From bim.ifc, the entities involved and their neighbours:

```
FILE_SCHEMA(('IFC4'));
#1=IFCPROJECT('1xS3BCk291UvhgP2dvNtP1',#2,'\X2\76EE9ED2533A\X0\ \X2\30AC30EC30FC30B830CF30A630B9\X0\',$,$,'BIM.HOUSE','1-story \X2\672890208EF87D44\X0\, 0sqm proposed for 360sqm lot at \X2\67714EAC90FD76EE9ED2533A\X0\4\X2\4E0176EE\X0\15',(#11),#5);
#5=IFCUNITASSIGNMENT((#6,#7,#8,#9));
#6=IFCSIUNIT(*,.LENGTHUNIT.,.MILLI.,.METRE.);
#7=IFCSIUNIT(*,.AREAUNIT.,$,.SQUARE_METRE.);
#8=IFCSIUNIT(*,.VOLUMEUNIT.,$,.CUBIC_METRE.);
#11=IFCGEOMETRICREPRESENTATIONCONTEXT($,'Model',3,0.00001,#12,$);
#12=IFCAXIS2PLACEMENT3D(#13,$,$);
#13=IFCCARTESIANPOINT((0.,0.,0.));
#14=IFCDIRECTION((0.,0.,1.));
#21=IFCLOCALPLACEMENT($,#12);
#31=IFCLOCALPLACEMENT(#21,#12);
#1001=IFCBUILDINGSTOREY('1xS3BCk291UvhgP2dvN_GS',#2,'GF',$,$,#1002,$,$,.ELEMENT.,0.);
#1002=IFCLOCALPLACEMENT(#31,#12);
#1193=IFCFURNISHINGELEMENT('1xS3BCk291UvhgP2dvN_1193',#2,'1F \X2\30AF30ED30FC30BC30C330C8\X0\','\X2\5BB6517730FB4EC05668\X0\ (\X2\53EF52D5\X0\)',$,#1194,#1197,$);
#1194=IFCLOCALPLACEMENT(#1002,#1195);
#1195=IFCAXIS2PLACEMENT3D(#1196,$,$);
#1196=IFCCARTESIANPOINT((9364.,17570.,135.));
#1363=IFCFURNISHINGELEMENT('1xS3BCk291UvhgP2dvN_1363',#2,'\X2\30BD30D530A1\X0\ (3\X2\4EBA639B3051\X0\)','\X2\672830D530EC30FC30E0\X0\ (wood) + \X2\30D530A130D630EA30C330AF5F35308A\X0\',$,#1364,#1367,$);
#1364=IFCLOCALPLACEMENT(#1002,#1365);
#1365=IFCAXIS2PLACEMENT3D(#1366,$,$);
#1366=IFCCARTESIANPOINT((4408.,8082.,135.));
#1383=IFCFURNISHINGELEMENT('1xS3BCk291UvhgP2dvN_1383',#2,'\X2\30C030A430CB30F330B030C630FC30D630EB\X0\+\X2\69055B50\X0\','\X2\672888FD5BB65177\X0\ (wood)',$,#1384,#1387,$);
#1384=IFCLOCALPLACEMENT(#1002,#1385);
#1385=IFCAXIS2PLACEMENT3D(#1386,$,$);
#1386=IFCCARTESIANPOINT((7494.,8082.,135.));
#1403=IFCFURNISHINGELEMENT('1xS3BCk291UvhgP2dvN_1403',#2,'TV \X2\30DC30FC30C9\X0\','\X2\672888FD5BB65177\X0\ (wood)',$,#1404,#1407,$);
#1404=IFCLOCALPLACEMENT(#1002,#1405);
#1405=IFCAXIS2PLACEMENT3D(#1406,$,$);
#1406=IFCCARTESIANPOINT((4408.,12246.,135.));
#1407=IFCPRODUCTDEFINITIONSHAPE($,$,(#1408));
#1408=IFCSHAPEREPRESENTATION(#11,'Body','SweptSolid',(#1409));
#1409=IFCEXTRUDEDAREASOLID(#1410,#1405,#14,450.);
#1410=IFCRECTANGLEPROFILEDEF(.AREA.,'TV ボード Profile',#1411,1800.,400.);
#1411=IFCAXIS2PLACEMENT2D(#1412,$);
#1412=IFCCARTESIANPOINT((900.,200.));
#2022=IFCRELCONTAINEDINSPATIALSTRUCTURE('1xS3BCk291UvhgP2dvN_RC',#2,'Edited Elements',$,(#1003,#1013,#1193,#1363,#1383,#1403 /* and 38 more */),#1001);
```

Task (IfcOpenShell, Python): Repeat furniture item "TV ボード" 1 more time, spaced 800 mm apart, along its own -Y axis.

```python
import ifcopenshell
import ifcopenshell.api.geometry
import ifcopenshell.api.root
import ifcopenshell.util.element
import ifcopenshell.util.placement

model = ifcopenshell.open("bim.ifc")


def reuse_history(source, copy):
    """copy_class also copies each property set's owner history, people and application; keep the originals."""
    for rel in copy.IsDefinedBy:
        if rel.is_a("IfcRelDefinesByProperties") and (history := rel.RelatingPropertyDefinition.OwnerHistory):
            rel.RelatingPropertyDefinition.OwnerHistory = source.OwnerHistory
            ifcopenshell.util.element.remove_deep2(model, history)


source = model.by_guid("1xS3BCk291UvhgP2dvN_1403")
base = ifcopenshell.util.placement.get_local_placement(source.ObjectPlacement)
step = -base[:3, 1] * 800.0

for i in range(1, 2):
    copy = ifcopenshell.api.root.copy_class(model, product=source)
    copy.Representation = ifcopenshell.util.element.copy_deep(
        model, source.Representation, exclude=["IfcGeometricRepresentationContext", "IfcRepresentationMap"]
    )
    reuse_history(source, copy)
    matrix = base.copy()
    matrix[:3, 3] += i * step
    print("added at", matrix[:3, 3].round(3) + 0.0)
    ifcopenshell.api.geometry.edit_object_placement(model, product=copy, matrix=matrix, is_si=False)

model.write("bim_updated.ifc")
```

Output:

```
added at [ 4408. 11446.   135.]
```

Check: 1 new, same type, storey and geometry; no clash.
